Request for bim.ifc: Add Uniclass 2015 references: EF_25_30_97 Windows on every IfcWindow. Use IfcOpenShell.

First a look at what the model holds.

```python
import ifcopenshell

model = ifcopenshell.open("bim.ifc")
print(model.schema)
print("classifications:", [c.Name for c in model.by_type("IfcClassification")])
for ifc_class in ("IfcDoor", "IfcRoof", "IfcStair", "IfcWall", "IfcWindow"):
    print(ifc_class, len(model.by_type(ifc_class)))
```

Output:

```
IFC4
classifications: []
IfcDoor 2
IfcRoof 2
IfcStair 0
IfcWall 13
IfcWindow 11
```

```python
import ifcopenshell
import ifcopenshell.api.classification

model = ifcopenshell.open("bim.ifc")

system = ifcopenshell.api.classification.add_classification(model, classification="Uniclass 2015")

codes = {
    "IfcWindow": ("EF_25_30_97", "Windows"),
}
for ifc_class, (code, name) in codes.items():
    products = model.by_type(ifc_class)
    ifcopenshell.api.classification.add_reference(
        model, products=products, classification=system, identification=code, name=name
    )
    print(code, len(products))

model.write("bim_rev.ifc")
```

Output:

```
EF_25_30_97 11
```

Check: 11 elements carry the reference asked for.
